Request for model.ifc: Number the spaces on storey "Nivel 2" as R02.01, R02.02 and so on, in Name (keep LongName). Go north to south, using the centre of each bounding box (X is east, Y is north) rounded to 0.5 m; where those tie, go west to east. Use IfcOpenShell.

First a look at what the model holds.

```python
import ifcopenshell
import ifcopenshell.util.element
import ifcopenshell.util.placement

model = ifcopenshell.open("model.ifc")
print(model.schema)
storey = next(s for s in model.by_type("IfcBuildingStorey") if s.Name == "Nivel 2")
spaces = [e for e in ifcopenshell.util.element.get_decomposition(storey) if e.is_a("IfcSpace")]
for e in sorted(spaces, key=lambda e: e.id()):
    origin = ifcopenshell.util.placement.get_local_placement(e.ObjectPlacement)[:3, 3]
    print(e.id(), e.Name, e.LongName, origin.round(2) + 0.0, sep=" | ")
```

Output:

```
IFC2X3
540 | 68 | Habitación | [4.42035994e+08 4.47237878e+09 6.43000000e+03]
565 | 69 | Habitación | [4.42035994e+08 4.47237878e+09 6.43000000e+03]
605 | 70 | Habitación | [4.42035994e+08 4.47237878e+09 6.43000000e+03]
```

```python
import ifcopenshell
import ifcopenshell.geom
import ifcopenshell.util.element
import ifcopenshell.util.shape

model = ifcopenshell.open("model.ifc")
settings = ifcopenshell.geom.settings()
settings.set("use-world-coords", True)


def centre(element):
    shape = ifcopenshell.geom.create_shape(settings, element)
    return ifcopenshell.util.shape.get_bbox_centroid(shape.geometry)


storey = next(s for s in model.by_type("IfcBuildingStorey") if s.Name == "Nivel 2")
spaces = [e for e in ifcopenshell.util.element.get_decomposition(storey) if e.is_a("IfcSpace")]

# Insertion points can sit at a corner or the storey origin, so sort by the geometry (in metres).
centres = {e: centre(e) for e in spaces}
spaces.sort(key=lambda e: (-round(centres[e][1] / 0.5), centres[e][0]))

for i, e in enumerate(spaces, start=1):
    number = f"R02.{i:02d}"
    e.Name = number
    print(e.id(), number)

model.write("model_edited.ifc")
```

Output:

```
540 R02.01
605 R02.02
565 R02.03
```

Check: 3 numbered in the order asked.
